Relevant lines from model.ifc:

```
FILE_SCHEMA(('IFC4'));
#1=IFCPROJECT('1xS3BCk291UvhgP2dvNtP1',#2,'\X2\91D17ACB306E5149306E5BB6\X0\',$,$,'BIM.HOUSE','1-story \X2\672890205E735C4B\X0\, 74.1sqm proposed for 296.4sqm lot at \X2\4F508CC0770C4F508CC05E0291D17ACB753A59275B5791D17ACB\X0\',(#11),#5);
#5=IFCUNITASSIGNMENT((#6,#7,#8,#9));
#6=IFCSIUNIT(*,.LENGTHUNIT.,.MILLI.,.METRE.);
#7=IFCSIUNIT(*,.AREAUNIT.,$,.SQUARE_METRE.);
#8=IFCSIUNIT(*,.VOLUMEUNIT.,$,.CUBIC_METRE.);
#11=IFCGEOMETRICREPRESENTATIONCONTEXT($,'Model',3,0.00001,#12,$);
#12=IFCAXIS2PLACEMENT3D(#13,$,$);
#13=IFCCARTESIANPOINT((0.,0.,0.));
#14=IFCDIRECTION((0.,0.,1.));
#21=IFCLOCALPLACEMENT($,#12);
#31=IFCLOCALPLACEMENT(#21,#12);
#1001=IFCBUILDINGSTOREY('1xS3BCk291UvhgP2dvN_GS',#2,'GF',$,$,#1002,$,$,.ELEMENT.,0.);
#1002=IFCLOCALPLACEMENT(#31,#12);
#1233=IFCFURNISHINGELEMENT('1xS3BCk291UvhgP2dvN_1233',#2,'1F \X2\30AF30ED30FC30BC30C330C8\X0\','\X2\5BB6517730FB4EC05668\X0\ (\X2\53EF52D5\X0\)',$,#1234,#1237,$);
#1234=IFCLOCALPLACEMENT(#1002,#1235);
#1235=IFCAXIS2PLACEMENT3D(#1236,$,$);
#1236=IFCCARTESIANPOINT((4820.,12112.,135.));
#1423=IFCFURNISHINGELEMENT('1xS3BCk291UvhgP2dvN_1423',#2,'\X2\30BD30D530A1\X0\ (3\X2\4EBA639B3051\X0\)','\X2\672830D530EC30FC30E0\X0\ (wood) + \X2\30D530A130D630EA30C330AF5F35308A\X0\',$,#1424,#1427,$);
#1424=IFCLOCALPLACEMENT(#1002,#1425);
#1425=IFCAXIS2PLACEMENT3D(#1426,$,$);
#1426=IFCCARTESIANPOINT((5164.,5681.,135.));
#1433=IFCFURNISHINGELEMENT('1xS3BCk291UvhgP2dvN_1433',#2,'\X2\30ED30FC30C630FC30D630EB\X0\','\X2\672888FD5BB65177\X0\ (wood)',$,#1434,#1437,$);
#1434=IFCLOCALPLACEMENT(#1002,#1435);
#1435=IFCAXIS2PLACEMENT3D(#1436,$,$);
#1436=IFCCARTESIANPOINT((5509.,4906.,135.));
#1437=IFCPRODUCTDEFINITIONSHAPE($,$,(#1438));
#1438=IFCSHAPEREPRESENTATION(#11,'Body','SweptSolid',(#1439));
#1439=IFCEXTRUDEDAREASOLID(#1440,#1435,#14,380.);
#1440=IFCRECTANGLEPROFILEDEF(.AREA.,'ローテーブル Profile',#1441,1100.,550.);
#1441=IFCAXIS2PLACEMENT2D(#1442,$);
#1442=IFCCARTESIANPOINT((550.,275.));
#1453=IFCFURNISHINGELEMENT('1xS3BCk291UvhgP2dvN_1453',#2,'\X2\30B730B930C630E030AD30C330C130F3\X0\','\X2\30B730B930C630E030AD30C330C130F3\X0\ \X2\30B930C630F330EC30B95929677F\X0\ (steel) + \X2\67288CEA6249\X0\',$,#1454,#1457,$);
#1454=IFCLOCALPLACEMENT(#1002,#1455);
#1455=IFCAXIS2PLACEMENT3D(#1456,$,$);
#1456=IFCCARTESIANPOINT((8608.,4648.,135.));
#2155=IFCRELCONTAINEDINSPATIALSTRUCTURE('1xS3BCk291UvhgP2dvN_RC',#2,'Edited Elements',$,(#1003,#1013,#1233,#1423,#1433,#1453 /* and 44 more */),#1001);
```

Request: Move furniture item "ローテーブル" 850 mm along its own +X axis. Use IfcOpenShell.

```python
import ifcopenshell
import ifcopenshell.api.geometry
import ifcopenshell.util.placement

model = ifcopenshell.open("model.ifc")

item = model.by_guid("1xS3BCk291UvhgP2dvN_1433")
matrix = ifcopenshell.util.placement.get_local_placement(item.ObjectPlacement)
matrix[:3, 3] += matrix[:3, 0] * 850.0
ifcopenshell.api.geometry.edit_object_placement(model, product=item, matrix=matrix, is_si=False)

print(ifcopenshell.util.placement.get_local_placement(item.ObjectPlacement).round(3) + 0.0)

model.write("model_rev.ifc")
```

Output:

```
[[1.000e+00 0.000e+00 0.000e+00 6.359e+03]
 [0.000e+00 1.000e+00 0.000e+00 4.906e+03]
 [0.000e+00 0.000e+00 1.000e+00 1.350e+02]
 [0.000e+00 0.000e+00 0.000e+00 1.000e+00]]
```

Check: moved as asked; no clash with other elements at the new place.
